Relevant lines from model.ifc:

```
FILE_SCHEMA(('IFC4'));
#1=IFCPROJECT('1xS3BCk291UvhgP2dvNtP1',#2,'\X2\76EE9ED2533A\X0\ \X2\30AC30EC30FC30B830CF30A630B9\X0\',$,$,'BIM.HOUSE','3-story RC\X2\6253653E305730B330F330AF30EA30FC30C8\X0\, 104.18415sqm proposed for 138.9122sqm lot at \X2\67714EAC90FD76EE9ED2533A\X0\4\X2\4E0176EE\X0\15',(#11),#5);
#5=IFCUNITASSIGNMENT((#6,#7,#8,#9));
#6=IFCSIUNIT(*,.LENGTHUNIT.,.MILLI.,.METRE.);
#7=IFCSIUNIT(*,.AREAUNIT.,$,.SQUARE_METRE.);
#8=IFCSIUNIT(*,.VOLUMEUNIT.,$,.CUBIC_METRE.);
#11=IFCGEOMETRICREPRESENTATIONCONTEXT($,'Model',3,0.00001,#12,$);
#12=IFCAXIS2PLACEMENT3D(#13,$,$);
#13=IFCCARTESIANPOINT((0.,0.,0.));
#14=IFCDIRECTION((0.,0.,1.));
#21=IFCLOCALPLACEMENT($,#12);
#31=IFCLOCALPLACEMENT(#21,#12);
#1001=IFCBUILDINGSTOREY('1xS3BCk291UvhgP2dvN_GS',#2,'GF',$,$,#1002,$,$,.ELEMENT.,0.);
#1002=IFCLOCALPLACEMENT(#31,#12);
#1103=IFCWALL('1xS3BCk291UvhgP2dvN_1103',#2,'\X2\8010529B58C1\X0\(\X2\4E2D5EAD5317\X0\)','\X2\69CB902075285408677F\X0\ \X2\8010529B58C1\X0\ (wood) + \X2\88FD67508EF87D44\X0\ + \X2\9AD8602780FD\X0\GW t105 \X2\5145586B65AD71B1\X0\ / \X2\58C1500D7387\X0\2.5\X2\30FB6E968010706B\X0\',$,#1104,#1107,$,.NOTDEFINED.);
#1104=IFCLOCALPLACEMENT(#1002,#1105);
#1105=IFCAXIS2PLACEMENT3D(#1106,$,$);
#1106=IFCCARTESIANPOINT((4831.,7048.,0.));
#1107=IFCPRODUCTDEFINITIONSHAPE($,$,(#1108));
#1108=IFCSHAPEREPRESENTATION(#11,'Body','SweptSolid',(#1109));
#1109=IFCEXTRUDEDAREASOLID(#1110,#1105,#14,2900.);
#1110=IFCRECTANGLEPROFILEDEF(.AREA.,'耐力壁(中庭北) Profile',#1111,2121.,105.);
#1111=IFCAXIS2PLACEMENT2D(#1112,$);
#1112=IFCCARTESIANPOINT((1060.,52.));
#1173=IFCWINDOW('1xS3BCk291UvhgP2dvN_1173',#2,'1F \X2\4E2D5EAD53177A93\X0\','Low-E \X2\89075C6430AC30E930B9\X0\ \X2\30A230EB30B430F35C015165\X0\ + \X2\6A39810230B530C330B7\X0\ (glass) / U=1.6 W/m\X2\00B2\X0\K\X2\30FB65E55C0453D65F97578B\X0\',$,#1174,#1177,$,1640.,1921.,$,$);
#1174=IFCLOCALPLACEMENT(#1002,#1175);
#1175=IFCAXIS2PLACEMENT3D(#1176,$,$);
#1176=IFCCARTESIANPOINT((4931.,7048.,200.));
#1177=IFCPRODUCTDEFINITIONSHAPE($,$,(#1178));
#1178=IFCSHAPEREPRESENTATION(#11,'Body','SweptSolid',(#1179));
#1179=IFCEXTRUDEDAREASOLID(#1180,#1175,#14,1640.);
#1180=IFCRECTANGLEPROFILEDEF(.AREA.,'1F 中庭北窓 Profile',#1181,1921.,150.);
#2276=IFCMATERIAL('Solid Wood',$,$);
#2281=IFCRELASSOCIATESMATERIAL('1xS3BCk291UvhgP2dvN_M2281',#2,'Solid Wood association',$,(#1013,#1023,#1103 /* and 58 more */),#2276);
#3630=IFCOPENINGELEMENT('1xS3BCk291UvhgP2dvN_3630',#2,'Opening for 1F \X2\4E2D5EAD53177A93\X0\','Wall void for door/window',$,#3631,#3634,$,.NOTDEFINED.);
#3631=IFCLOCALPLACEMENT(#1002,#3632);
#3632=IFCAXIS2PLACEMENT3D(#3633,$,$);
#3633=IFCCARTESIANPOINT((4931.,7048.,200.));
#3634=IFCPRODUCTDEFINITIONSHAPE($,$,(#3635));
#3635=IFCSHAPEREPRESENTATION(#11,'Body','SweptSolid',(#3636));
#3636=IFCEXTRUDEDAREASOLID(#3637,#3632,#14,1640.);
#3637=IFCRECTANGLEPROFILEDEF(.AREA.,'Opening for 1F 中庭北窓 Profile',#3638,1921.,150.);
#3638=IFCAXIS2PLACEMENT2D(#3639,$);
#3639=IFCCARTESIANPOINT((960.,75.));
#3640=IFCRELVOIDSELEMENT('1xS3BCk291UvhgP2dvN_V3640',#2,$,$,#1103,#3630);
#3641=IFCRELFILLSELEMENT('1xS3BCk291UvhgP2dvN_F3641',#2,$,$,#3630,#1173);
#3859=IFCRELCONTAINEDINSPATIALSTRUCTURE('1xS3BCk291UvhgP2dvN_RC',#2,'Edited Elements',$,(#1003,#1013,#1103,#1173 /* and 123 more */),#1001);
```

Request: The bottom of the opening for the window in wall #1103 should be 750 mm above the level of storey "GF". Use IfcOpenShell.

```python
import numpy as np
import ifcopenshell
import ifcopenshell.api.geometry
import ifcopenshell.geom
import ifcopenshell.util.element
import ifcopenshell.util.placement
import ifcopenshell.util.shape
import ifcopenshell.util.unit

model = ifcopenshell.open("model.ifc")
unit_scale = ifcopenshell.util.unit.calculate_unit_scale(model)

window = model.by_guid("1xS3BCk291UvhgP2dvN_1173")
opening = window.FillsVoids[0].RelatingOpeningElement
storey = ifcopenshell.util.element.get_container(window, ifc_class="IfcBuildingStorey")
level = ifcopenshell.util.placement.get_local_placement(storey.ObjectPlacement)[2, 3]

# The opening's origin need not be at the sill, so measure its lowest point.
shape = ifcopenshell.geom.create_shape(ifcopenshell.geom.settings(), opening)
bottom = ifcopenshell.util.shape.get_shape_bottom_elevation(shape, shape.geometry) / unit_scale
dz = level + 0.75 / unit_scale - bottom

shift = np.array([0.0, 0.0, dz])
# The window is not placed relative to its opening, so move both.
for product in (opening, window):
    matrix = ifcopenshell.util.placement.get_local_placement(product.ObjectPlacement)
    matrix[:3, 3] += shift
    ifcopenshell.api.geometry.edit_object_placement(model, product=product, matrix=matrix, is_si=False)

print(f"moved by {dz * unit_scale:+.3f} m")

model.write("model_v2.ifc")
```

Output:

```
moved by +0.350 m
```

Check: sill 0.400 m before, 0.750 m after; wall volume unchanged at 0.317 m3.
